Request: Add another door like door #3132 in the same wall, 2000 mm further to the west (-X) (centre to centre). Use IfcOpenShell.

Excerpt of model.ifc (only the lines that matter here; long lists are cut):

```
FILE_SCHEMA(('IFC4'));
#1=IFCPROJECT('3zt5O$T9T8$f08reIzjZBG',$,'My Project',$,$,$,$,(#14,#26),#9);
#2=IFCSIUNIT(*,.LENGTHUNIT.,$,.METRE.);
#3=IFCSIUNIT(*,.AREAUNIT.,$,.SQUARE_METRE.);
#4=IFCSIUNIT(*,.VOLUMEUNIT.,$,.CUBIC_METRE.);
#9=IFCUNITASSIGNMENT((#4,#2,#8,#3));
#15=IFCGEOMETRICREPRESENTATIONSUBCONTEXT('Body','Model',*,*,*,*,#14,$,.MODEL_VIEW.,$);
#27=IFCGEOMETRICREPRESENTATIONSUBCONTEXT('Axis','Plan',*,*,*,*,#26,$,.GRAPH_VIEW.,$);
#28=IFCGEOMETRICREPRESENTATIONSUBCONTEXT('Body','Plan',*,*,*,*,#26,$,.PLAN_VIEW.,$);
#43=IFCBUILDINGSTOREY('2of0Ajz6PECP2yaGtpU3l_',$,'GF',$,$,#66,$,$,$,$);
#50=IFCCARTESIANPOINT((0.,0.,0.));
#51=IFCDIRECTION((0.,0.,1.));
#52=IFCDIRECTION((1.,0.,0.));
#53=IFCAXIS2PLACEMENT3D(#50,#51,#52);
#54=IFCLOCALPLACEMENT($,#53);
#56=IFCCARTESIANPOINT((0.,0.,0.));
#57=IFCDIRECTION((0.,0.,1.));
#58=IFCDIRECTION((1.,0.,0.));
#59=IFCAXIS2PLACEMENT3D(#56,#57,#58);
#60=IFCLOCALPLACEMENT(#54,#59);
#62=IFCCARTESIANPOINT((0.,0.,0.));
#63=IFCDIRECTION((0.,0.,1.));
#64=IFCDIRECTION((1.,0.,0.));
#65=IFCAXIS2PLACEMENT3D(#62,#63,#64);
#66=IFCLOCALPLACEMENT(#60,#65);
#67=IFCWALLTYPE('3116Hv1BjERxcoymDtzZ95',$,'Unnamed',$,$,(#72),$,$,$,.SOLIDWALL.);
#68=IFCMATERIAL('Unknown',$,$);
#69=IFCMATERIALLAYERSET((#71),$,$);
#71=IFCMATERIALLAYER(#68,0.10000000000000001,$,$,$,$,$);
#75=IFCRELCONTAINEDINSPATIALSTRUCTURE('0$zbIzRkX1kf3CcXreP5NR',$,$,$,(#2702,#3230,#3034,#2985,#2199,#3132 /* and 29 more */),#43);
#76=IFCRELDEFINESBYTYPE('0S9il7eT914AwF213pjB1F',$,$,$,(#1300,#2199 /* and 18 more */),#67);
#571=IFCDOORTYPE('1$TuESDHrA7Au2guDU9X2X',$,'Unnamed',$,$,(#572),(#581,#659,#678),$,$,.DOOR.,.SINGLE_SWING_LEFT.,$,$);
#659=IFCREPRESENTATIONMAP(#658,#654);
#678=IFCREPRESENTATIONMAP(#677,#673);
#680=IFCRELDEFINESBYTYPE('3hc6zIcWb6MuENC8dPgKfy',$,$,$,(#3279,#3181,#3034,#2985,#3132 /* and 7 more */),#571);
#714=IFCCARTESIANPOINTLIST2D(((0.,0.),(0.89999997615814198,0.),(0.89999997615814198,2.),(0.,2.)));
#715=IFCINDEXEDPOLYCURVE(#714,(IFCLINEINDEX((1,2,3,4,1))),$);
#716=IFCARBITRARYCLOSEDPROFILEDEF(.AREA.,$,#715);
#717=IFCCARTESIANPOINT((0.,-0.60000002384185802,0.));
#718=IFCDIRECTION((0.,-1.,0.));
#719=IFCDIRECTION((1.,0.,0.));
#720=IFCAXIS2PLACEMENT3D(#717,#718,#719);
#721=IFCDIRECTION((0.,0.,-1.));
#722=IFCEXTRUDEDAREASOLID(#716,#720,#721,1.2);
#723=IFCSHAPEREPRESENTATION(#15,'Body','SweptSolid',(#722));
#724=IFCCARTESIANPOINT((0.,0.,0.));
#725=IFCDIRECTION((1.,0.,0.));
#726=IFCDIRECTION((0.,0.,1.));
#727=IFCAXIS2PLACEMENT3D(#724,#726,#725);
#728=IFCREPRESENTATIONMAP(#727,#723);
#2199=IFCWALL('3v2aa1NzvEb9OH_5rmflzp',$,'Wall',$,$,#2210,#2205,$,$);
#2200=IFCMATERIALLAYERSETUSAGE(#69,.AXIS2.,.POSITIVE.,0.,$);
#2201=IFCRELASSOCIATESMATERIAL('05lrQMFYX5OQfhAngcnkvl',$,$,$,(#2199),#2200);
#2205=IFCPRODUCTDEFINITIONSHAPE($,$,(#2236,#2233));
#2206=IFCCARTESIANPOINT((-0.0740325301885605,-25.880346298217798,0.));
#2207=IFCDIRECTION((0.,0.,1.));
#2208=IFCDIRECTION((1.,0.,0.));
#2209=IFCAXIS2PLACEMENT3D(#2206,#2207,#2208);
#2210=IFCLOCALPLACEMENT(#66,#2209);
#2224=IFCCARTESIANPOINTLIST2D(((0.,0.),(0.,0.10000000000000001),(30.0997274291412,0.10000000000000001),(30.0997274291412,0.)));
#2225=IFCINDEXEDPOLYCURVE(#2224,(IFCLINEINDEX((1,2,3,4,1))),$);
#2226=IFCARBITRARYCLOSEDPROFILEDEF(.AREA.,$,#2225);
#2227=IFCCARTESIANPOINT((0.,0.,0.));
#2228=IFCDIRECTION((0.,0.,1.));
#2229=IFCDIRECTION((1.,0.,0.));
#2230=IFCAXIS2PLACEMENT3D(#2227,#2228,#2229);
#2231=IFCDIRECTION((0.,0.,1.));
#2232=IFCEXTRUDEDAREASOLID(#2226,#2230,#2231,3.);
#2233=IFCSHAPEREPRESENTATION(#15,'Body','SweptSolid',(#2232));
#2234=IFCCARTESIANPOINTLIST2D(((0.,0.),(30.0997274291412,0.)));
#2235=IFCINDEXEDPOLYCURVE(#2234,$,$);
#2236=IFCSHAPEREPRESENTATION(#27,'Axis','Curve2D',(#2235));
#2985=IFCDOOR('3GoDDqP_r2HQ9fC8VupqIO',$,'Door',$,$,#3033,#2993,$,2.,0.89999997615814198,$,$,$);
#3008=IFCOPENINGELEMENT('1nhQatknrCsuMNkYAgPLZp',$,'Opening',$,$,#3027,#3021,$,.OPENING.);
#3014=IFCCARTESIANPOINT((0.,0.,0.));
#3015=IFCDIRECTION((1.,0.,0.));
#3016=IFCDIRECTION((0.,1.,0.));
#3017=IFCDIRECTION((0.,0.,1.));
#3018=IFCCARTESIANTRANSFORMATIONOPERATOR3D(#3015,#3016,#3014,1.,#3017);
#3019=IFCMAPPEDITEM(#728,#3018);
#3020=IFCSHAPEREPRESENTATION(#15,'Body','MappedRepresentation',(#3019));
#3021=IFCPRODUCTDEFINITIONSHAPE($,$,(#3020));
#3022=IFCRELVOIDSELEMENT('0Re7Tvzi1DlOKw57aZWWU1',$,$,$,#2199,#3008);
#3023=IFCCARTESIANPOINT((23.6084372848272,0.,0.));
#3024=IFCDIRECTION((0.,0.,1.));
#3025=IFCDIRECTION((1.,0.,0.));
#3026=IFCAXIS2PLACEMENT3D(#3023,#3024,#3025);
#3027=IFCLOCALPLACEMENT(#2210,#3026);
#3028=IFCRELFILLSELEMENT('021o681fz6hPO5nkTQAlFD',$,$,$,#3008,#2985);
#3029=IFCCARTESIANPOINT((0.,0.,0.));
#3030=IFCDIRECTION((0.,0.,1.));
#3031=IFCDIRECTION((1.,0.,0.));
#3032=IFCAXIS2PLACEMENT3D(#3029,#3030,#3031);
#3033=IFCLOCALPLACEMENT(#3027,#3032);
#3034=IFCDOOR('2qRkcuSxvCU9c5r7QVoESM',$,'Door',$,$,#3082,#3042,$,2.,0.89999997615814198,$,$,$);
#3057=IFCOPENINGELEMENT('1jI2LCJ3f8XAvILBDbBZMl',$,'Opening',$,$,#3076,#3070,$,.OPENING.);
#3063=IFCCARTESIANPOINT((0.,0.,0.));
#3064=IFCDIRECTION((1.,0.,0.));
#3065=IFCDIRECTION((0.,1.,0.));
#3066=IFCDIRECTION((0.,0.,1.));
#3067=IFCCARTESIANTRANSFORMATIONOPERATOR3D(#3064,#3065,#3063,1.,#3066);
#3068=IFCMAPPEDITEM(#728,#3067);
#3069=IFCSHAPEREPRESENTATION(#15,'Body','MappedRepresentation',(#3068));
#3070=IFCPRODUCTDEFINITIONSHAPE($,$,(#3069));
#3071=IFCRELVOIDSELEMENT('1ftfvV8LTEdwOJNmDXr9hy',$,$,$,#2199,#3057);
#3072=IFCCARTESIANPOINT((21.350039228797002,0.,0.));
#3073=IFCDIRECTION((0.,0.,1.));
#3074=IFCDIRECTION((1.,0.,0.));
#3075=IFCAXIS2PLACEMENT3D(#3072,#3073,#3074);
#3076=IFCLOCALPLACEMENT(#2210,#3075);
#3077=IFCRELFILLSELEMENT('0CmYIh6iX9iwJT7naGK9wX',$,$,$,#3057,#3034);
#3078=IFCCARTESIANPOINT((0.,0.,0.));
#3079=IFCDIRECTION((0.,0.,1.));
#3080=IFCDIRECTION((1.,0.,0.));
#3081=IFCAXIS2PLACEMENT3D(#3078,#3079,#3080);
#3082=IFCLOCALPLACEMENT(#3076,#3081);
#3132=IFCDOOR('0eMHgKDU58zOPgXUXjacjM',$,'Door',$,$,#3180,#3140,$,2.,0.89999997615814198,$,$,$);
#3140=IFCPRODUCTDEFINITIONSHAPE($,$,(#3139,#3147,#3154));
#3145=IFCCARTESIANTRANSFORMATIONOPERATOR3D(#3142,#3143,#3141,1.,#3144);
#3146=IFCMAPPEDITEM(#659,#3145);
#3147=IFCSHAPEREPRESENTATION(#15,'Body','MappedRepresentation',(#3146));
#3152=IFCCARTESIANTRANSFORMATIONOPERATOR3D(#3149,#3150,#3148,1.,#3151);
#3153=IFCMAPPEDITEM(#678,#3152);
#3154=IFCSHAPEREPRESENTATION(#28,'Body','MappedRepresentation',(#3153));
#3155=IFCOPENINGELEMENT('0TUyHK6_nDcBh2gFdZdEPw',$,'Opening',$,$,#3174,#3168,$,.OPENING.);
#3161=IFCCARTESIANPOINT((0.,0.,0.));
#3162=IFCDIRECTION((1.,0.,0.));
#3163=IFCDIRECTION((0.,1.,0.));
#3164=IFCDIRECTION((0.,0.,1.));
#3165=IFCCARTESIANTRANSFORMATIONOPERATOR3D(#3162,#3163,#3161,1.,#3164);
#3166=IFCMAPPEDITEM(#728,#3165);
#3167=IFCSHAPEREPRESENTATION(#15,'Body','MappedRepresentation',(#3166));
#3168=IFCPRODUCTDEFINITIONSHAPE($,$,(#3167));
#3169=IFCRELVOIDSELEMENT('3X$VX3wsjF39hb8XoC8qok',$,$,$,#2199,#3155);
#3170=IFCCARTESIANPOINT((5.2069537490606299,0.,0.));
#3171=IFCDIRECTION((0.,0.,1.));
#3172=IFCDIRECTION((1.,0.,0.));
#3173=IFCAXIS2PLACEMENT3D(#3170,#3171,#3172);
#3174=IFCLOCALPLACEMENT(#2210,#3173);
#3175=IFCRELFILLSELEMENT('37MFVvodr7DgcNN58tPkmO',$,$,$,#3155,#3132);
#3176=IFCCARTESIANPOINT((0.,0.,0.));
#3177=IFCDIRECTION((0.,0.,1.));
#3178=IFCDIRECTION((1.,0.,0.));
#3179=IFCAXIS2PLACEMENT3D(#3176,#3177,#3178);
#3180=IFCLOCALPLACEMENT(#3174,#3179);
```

```python
import ifcopenshell
import ifcopenshell.api.feature
import ifcopenshell.api.geometry
import ifcopenshell.api.root
import ifcopenshell.geom
import ifcopenshell.util.element
import ifcopenshell.util.placement
import ifcopenshell.util.shape
import ifcopenshell.util.unit

model = ifcopenshell.open("model.ifc")
unit_scale = ifcopenshell.util.unit.calculate_unit_scale(model)
settings = ifcopenshell.geom.settings()


def volume(element):
    """Net volume in cubic metres, openings subtracted."""
    shape = ifcopenshell.geom.create_shape(settings, element)
    return ifcopenshell.util.shape.get_volume(shape.geometry)


door = model.by_guid("0eMHgKDU58zOPgXUXjacjM")
opening = door.FillsVoids[0].RelatingOpeningElement
wall = opening.VoidsElements[0].RelatingBuildingElement
before = volume(wall)
shift = ifcopenshell.util.placement.get_local_placement(wall.ObjectPlacement)[:3, 0] * -2 / unit_scale

# copy_class copies the void relationship, type, container and properties, but no geometry.
new_opening = ifcopenshell.api.root.copy_class(model, product=opening)
new_opening.Representation = ifcopenshell.util.element.copy_deep(
    model, opening.Representation, exclude=["IfcGeometricRepresentationContext", "IfcRepresentationMap"]
)
new_door = ifcopenshell.api.root.copy_class(model, product=door)
new_door.Representation = ifcopenshell.util.element.copy_deep(
    model, door.Representation, exclude=["IfcGeometricRepresentationContext", "IfcRepresentationMap"]
)
ifcopenshell.api.feature.add_filling(model, opening=new_opening, element=new_door)

for old, new in ((opening, new_opening), (door, new_door)):
    matrix = ifcopenshell.util.placement.get_local_placement(old.ObjectPlacement)
    matrix[:3, 3] += shift
    ifcopenshell.api.geometry.edit_object_placement(model, product=new, matrix=matrix, is_si=False)

after = volume(wall)

print(f"wall volume {before:.3f} -> {after:.3f} m3")

model.write("model_updated.ifc")
```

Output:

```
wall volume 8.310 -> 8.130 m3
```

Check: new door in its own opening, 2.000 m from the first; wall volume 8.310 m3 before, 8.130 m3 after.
